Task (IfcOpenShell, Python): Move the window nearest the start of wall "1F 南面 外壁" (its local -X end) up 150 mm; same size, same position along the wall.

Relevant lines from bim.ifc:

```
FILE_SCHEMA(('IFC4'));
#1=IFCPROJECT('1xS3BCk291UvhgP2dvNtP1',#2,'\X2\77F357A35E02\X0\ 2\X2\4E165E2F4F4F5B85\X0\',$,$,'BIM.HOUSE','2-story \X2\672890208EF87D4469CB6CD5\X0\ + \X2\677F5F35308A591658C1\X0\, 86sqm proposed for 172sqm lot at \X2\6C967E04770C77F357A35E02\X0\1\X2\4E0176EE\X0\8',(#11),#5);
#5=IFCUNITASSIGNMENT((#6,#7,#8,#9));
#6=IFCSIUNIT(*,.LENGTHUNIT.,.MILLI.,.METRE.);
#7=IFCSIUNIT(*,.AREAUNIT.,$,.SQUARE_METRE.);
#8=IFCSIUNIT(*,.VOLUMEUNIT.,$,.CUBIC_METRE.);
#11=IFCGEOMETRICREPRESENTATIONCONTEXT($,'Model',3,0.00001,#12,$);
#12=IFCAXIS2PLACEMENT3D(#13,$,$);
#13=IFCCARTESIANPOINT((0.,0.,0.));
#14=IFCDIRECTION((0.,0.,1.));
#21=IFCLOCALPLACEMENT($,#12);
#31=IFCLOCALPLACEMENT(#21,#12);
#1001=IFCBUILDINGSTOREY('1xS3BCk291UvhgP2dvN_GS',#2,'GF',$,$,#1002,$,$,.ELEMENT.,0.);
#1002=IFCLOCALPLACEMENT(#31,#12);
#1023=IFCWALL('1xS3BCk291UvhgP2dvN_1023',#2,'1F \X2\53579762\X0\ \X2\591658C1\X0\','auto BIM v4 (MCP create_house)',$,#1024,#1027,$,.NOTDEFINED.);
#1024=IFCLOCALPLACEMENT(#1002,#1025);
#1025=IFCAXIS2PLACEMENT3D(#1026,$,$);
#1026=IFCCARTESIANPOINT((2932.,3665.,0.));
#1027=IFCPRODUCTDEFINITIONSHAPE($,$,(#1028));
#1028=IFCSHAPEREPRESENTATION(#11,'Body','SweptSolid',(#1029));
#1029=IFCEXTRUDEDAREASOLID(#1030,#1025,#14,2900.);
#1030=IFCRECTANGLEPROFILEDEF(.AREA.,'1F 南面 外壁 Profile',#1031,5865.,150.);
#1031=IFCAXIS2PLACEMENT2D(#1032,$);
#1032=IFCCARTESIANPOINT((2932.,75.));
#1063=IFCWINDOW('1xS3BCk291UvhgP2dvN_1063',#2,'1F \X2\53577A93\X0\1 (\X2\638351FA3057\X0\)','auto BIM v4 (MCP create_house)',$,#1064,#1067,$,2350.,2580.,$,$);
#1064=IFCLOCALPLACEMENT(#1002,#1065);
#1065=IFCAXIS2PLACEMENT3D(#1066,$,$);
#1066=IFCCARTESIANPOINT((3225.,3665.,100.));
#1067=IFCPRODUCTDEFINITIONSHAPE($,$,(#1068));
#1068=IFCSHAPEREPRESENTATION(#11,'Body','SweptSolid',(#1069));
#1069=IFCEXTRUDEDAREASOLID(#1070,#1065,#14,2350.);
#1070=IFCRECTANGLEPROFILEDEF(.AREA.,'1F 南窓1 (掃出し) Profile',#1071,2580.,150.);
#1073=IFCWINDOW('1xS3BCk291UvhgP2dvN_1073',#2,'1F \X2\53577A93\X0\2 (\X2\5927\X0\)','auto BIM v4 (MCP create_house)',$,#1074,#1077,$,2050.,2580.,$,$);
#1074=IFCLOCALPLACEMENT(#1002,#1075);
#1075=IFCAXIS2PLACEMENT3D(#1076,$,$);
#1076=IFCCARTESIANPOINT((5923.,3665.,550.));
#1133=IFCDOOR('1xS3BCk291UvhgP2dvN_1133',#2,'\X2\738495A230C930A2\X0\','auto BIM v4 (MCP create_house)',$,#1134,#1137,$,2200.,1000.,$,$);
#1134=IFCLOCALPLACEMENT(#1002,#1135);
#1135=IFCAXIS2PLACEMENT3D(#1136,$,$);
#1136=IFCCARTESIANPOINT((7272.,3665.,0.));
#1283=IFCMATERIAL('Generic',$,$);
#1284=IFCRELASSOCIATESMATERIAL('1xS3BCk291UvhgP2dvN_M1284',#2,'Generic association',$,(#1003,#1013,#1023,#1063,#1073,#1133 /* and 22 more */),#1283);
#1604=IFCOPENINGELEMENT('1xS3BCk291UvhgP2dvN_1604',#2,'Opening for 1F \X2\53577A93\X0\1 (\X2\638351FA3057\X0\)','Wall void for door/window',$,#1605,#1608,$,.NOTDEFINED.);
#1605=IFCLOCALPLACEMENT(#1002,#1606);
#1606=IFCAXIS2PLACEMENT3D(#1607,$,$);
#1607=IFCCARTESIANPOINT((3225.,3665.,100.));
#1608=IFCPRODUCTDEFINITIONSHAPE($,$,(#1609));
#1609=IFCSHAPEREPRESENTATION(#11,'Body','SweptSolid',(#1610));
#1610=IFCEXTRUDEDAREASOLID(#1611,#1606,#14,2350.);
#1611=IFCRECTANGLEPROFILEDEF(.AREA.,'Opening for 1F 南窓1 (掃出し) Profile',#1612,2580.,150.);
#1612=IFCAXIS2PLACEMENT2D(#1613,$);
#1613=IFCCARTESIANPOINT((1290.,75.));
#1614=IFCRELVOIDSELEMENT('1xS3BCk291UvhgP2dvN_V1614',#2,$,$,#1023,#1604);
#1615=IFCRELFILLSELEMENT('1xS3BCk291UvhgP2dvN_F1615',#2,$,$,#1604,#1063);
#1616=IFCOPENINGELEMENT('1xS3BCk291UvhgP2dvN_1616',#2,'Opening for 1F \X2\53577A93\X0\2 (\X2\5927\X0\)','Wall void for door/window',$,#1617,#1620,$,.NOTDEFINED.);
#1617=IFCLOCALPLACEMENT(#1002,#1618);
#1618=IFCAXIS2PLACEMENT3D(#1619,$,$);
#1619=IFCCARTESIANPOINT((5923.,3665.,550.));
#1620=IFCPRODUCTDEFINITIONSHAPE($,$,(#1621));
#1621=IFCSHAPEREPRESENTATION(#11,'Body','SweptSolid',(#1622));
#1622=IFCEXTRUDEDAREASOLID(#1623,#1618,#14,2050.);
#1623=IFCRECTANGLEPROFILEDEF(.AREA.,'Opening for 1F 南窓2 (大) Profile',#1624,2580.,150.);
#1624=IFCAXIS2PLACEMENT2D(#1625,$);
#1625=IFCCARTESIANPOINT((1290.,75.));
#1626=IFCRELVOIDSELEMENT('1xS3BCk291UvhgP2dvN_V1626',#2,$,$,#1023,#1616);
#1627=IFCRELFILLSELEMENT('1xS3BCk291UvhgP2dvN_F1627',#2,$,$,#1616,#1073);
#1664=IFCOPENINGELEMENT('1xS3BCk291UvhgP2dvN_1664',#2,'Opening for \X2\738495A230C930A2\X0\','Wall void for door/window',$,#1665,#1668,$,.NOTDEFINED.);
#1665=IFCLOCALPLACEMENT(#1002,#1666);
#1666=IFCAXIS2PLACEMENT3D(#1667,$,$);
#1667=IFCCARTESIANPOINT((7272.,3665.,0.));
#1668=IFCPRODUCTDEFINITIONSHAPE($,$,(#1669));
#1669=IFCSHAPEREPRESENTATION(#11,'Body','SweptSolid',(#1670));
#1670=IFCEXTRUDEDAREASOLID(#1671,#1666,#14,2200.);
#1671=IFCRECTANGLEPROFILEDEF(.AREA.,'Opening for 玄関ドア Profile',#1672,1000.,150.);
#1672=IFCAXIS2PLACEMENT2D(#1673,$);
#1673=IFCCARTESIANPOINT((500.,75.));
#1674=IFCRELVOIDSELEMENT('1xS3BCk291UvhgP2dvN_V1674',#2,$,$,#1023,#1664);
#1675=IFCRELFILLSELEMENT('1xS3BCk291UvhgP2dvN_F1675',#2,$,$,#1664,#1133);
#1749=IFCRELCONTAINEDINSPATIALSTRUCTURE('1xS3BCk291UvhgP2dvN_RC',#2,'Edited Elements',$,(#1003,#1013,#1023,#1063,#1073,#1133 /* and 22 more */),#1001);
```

```python
import numpy as np
import ifcopenshell
import ifcopenshell.api.geometry
import ifcopenshell.util.placement
import ifcopenshell.util.unit

model = ifcopenshell.open("bim.ifc")
unit_scale = ifcopenshell.util.unit.calculate_unit_scale(model)

window = model.by_guid("1xS3BCk291UvhgP2dvN_1063")
opening = window.FillsVoids[0].RelatingOpeningElement
dz = 150.0

shift = np.array([0.0, 0.0, dz])
# The window is not placed relative to its opening, so move both.
for product in (opening, window):
    matrix = ifcopenshell.util.placement.get_local_placement(product.ObjectPlacement)
    matrix[:3, 3] += shift
    ifcopenshell.api.geometry.edit_object_placement(model, product=product, matrix=matrix, is_si=False)

print(f"moved by {dz * unit_scale:+.3f} m")

model.write("bim_rev.ifc")
```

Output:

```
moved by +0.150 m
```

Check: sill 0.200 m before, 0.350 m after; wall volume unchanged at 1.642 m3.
